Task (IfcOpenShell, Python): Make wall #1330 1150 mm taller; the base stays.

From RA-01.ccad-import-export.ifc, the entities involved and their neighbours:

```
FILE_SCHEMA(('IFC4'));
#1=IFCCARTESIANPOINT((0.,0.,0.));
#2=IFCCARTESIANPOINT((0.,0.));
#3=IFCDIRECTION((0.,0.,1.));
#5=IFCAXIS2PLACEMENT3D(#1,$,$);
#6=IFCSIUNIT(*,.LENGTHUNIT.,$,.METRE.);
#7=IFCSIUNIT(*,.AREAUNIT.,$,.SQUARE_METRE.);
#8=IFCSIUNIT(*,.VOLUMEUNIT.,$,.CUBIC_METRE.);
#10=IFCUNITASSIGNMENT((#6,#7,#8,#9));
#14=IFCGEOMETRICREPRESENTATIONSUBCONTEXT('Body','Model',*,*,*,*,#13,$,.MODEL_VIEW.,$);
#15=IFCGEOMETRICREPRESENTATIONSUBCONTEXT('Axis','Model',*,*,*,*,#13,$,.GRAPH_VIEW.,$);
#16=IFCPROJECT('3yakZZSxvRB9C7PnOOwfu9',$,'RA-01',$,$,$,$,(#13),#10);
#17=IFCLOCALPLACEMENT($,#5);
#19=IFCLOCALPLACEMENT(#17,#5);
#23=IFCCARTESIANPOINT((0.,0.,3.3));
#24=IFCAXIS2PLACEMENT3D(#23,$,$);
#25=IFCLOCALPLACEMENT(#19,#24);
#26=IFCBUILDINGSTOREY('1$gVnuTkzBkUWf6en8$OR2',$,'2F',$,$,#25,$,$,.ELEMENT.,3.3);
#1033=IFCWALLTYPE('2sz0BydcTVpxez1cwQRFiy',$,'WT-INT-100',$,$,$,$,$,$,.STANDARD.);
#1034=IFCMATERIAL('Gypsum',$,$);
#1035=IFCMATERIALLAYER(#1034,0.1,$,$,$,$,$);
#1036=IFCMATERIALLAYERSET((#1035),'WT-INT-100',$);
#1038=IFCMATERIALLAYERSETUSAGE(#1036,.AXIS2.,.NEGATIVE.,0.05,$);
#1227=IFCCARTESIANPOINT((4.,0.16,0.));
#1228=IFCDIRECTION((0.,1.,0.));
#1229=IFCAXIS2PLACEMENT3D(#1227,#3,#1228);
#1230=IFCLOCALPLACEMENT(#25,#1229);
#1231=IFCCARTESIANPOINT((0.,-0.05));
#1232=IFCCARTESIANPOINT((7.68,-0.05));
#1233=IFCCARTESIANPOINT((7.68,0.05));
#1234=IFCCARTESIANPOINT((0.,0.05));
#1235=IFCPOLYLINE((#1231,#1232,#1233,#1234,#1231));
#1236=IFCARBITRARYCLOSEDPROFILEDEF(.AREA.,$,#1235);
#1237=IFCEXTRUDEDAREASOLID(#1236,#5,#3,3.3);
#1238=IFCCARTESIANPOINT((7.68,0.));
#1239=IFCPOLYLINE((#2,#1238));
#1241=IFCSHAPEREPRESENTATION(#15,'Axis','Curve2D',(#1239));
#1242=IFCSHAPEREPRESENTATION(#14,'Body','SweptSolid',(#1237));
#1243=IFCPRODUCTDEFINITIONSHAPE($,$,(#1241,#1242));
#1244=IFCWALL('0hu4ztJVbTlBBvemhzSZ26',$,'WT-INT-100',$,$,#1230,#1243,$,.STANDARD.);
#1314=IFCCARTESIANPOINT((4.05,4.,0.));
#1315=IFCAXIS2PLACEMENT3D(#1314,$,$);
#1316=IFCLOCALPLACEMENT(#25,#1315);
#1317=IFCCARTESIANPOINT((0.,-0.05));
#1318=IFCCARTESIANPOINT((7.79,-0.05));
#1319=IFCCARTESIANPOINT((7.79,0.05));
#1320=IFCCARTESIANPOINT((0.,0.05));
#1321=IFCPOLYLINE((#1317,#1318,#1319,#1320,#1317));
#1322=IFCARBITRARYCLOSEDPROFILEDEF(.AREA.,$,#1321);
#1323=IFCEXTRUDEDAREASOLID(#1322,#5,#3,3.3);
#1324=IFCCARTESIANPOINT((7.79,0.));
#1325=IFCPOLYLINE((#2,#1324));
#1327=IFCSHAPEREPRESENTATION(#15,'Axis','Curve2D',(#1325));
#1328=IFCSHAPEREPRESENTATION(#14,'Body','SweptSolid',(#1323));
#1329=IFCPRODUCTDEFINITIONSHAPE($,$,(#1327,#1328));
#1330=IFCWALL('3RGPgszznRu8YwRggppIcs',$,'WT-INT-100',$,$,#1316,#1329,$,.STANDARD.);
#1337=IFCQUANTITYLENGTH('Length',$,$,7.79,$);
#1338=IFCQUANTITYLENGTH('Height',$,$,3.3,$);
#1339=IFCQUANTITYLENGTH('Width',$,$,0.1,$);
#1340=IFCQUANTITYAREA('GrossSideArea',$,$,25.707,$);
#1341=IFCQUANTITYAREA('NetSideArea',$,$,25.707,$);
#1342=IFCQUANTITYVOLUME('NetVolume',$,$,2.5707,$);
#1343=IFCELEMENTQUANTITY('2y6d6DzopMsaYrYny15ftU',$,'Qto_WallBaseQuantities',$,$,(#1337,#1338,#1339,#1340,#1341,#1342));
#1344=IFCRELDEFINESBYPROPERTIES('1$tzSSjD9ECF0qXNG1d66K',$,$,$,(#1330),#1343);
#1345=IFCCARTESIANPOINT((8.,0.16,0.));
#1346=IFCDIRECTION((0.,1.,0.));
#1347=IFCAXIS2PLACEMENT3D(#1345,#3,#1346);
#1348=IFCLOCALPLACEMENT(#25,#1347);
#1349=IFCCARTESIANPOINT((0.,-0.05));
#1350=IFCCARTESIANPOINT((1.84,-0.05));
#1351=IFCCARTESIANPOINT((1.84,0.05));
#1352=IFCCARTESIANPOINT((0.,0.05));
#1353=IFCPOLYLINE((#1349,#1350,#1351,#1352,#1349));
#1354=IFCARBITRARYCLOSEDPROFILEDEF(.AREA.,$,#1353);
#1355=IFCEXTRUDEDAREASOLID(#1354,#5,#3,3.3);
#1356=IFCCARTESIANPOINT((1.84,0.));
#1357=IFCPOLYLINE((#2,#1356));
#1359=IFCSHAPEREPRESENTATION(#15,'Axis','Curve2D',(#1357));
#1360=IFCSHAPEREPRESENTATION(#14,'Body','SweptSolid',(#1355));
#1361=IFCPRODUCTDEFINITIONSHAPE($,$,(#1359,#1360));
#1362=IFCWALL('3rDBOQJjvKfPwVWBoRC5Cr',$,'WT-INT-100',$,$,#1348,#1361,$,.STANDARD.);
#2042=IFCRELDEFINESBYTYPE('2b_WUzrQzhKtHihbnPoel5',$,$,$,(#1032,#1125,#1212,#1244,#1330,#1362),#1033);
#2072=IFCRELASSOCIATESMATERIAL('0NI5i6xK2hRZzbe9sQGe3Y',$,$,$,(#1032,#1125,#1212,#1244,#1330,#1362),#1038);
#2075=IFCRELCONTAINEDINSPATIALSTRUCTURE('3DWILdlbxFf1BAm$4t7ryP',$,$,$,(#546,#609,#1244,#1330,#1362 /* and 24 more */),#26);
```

```python
import ifcopenshell
import ifcopenshell.api.pset
import ifcopenshell.geom
import ifcopenshell.util.element
import ifcopenshell.util.representation
import ifcopenshell.util.shape
import ifcopenshell.util.unit

model = ifcopenshell.open("RA-01.ccad-import-export.ifc")
unit_scale = ifcopenshell.util.unit.calculate_unit_scale(model)
area_scale = ifcopenshell.util.unit.calculate_unit_scale(model, "AREAUNIT")
volume_scale = ifcopenshell.util.unit.calculate_unit_scale(model, "VOLUMEUNIT")
settings = ifcopenshell.geom.settings()


def volume(element):
    """Net volume in cubic metres, openings subtracted."""
    shape = ifcopenshell.geom.create_shape(settings, element)
    return ifcopenshell.util.shape.get_volume(shape.geometry)


wall = model.by_guid("3RGPgszznRu8YwRggppIcs")
before = volume(wall)

body = ifcopenshell.util.representation.get_representation(wall, "Model", "Body")
solid = body.Items[0]
old_height = solid.Depth
solid.Depth += 1.15
after = volume(wall)
thickness = 0.1  # wall thickness in metres

# Update the stored height, areas and volumes.
qto = model.by_id(ifcopenshell.util.element.get_pset(wall, "Qto_WallBaseQuantities", should_inherit=False)["id"])
ifcopenshell.api.pset.edit_qto(model, qto=qto, properties={
    "Height": solid.Depth,
    "GrossSideArea": ifcopenshell.util.element.get_pset(wall, "Qto_WallBaseQuantities", "GrossSideArea") * solid.Depth / old_height,
    "NetSideArea": after / thickness / area_scale,
    "NetVolume": after / volume_scale,
})

print(f"height {old_height:g} -> {solid.Depth:g}, volume {before:.3f} -> {after:.3f} m3")

model.write("RA-01.ccad-import-export-out.ifc")
```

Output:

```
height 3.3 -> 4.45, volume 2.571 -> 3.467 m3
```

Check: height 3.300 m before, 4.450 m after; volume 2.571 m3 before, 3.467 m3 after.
